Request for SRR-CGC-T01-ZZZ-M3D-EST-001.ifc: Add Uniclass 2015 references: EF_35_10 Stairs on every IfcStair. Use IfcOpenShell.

First a look at what the model holds.

```python
import ifcopenshell

model = ifcopenshell.open("SRR-CGC-T01-ZZZ-M3D-EST-001.ifc")
print(model.schema)
print("classifications:", [c.Name for c in model.by_type("IfcClassification")])
for ifc_class in ("IfcDoor", "IfcRoof", "IfcStair", "IfcWall", "IfcWindow"):
    print(ifc_class, len(model.by_type(ifc_class)))
```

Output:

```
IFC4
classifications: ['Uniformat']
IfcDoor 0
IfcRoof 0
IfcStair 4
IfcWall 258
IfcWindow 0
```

```python
import ifcopenshell
import ifcopenshell.api.classification

model = ifcopenshell.open("SRR-CGC-T01-ZZZ-M3D-EST-001.ifc")

system = ifcopenshell.api.classification.add_classification(model, classification="Uniclass 2015")

codes = {
    "IfcStair": ("EF_35_10", "Stairs"),
}
for ifc_class, (code, name) in codes.items():
    products = model.by_type(ifc_class)
    ifcopenshell.api.classification.add_reference(
        model, products=products, classification=system, identification=code, name=name
    )
    print(code, len(products))

model.write("SRR-CGC-T01-ZZZ-M3D-EST-001_rev.ifc")
```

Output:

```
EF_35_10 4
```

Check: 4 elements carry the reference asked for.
